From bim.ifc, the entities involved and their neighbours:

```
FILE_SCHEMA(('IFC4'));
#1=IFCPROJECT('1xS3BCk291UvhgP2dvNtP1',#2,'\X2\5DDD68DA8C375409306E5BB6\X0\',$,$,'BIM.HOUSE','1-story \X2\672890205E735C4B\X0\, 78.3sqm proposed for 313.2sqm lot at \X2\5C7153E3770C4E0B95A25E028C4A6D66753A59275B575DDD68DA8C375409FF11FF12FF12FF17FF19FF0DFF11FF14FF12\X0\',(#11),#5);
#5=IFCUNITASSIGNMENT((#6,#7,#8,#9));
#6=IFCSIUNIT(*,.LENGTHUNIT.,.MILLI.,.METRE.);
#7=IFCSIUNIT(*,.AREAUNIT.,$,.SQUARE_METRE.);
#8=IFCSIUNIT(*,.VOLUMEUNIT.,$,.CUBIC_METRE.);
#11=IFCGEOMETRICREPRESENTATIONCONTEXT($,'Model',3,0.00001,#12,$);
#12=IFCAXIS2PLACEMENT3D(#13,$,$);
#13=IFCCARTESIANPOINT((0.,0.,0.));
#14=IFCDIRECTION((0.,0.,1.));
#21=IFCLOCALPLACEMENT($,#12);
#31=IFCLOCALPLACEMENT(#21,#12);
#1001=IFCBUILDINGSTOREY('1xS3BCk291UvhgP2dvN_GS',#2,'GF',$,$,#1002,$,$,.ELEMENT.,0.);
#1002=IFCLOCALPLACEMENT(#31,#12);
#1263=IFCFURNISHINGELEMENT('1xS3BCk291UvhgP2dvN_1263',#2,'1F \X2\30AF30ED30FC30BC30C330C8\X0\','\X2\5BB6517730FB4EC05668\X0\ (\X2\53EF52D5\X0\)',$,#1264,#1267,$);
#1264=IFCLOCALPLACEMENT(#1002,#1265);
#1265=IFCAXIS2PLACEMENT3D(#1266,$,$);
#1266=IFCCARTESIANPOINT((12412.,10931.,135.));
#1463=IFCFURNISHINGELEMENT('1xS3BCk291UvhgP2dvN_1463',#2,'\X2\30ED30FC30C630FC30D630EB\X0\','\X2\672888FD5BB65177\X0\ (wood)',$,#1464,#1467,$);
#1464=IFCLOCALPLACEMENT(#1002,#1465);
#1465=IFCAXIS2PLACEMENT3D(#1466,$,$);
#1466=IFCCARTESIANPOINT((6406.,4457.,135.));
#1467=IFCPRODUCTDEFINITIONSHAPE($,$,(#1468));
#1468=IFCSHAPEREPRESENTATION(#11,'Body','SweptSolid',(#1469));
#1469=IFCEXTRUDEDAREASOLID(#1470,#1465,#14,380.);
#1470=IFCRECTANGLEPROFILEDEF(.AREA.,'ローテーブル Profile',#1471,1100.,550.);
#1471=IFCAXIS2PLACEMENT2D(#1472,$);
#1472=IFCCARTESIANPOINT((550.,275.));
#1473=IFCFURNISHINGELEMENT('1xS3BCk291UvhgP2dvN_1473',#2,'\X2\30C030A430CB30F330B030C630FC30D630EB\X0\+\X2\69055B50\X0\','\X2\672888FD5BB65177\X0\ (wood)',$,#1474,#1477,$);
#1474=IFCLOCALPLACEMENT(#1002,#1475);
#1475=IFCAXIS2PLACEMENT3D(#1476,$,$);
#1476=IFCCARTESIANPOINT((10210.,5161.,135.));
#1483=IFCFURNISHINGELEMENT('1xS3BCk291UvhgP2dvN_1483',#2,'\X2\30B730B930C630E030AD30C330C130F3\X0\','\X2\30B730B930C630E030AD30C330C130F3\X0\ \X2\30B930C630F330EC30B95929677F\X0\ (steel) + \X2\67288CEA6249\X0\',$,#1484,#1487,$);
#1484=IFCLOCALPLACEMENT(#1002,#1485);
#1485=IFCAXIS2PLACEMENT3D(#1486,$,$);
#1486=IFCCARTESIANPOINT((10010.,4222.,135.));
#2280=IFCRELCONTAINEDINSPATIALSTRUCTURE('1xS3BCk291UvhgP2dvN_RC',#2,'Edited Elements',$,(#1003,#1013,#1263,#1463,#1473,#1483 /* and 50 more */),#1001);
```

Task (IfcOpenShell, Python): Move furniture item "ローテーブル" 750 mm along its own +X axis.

```python
import ifcopenshell
import ifcopenshell.api.geometry
import ifcopenshell.util.placement

model = ifcopenshell.open("bim.ifc")

item = model.by_guid("1xS3BCk291UvhgP2dvN_1463")
matrix = ifcopenshell.util.placement.get_local_placement(item.ObjectPlacement)
matrix[:3, 3] += matrix[:3, 0] * 750.0
ifcopenshell.api.geometry.edit_object_placement(model, product=item, matrix=matrix, is_si=False)

print(ifcopenshell.util.placement.get_local_placement(item.ObjectPlacement).round(3) + 0.0)

model.write("bim-out.ifc")
```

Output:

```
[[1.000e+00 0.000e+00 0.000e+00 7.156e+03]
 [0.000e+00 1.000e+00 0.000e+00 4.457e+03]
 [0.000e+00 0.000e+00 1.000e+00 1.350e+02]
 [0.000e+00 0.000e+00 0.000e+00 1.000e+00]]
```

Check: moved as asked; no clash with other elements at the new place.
